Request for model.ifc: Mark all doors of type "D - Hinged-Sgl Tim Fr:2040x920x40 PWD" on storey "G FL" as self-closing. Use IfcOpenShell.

First a look at what the model holds.

```python
import ifcopenshell
import ifcopenshell.util.element

model = ifcopenshell.open("model.ifc")
print(model.schema)
storey = next(s for s in model.by_type("IfcBuildingStorey") if s.Name == "G FL")
doors = [e for e in ifcopenshell.util.element.get_decomposition(storey) if e.is_a("IfcDoor")]
seen = {}
for e in doors:
    element_type = ifcopenshell.util.element.get_type(e)
    key = (element_type.Name if element_type != e and element_type else None, ifcopenshell.util.element.get_pset(e, "Pset_DoorCommon", "SelfClosing"))
    seen[key] = seen.get(key, 0) + 1
for (name, value), count in sorted(seen.items(), key=str):
    print(count, "x", name, "|", value)
```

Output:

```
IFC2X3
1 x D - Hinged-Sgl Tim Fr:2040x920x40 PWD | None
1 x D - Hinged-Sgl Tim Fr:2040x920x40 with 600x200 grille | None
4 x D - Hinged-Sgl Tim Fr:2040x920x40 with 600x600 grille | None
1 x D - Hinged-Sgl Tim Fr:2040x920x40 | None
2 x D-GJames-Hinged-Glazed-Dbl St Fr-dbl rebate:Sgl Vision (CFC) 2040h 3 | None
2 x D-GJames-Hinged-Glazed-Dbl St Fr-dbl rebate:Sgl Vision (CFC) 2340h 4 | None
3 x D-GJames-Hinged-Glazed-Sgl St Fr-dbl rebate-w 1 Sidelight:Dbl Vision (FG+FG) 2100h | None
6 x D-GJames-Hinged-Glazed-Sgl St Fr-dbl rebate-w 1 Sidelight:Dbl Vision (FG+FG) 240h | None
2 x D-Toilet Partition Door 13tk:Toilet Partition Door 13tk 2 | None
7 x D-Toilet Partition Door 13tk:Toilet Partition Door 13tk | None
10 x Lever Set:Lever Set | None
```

```python
import ifcopenshell
import ifcopenshell.api.pset
import ifcopenshell.util.element

model = ifcopenshell.open("model.ifc")

storey = next(s for s in model.by_type("IfcBuildingStorey") if s.Name == "G FL")
doors = [e for e in ifcopenshell.util.element.get_decomposition(storey) if e.is_a("IfcDoor")]

count = 0
for e in doors:
    element_type = ifcopenshell.util.element.get_type(e)
    if element_type in (None, e) or element_type.Name != "D - Hinged-Sgl Tim Fr:2040x920x40 PWD":
        continue
    # add_pset returns the element's existing set when there is one.
    pset = ifcopenshell.api.pset.add_pset(model, product=e, name="Pset_DoorCommon")
    ifcopenshell.api.pset.edit_pset(model, pset=pset, properties={"SelfClosing": True})
    count += 1

print(count, "doors updated")

model.write("model_updated.ifc")
```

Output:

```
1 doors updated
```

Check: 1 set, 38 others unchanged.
